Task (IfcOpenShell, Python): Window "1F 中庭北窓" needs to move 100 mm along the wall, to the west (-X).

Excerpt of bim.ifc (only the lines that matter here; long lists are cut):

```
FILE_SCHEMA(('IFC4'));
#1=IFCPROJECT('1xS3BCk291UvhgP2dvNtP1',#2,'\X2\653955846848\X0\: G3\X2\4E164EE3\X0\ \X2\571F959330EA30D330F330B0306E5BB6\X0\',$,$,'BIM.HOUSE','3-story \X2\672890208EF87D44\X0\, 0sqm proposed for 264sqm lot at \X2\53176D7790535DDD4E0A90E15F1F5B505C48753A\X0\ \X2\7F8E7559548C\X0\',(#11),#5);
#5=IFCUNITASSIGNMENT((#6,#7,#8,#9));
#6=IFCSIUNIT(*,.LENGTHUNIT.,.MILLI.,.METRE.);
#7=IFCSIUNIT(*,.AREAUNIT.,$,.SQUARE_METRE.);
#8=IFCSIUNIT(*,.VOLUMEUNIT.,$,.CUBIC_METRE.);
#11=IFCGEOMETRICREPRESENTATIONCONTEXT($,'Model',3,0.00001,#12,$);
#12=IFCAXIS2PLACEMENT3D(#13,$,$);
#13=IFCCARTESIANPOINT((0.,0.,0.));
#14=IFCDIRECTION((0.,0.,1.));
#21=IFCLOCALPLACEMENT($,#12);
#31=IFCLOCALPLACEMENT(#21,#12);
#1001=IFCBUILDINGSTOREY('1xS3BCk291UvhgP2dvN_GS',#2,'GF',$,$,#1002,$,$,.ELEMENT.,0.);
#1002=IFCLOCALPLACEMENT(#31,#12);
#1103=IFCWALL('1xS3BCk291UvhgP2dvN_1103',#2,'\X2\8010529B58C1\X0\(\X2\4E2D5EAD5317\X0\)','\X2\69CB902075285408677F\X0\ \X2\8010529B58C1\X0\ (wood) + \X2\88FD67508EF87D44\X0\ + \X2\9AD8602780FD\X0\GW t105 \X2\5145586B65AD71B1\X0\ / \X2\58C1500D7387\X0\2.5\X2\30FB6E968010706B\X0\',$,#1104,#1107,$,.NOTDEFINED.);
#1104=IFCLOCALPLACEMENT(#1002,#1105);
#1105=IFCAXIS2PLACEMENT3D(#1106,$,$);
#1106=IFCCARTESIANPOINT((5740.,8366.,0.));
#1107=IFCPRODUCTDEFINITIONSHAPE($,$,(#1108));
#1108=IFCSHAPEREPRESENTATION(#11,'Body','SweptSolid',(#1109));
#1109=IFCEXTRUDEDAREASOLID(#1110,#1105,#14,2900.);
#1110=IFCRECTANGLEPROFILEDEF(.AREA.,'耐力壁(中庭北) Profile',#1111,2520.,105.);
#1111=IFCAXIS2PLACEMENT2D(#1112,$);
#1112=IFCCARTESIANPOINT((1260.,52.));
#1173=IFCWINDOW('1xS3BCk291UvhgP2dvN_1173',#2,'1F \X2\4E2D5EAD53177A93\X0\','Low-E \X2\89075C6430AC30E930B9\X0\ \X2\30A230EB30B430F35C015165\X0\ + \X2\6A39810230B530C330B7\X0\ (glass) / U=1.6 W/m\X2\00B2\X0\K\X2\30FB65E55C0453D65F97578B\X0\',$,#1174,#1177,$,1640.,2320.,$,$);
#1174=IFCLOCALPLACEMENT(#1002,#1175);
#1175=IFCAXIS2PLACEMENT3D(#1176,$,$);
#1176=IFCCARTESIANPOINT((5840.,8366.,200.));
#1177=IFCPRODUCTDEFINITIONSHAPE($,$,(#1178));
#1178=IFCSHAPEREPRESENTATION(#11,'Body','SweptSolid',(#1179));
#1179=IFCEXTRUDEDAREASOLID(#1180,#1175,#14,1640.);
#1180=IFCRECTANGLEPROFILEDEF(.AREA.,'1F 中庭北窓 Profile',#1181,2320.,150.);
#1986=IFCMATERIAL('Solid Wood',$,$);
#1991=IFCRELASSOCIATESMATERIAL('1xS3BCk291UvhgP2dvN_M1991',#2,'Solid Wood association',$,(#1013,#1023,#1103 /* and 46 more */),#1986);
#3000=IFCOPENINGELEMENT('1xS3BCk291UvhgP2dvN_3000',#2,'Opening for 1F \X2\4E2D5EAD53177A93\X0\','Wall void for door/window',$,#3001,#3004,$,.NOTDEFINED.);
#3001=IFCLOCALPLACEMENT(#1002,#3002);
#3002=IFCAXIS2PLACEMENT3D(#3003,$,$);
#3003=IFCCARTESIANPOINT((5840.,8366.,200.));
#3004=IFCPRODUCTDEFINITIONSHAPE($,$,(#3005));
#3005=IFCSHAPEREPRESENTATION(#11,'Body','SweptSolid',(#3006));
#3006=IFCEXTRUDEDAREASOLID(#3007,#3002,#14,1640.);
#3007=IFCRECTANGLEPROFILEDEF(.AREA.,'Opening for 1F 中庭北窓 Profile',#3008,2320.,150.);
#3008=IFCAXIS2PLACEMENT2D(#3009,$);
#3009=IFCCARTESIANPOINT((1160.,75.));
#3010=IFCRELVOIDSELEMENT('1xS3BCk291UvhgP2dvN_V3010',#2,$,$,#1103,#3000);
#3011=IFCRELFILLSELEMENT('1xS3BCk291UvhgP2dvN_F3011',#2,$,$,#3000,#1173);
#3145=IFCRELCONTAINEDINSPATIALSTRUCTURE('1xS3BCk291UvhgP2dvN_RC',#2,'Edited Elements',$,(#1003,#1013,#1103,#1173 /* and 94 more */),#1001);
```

```python
import ifcopenshell
import ifcopenshell.api.geometry
import ifcopenshell.util.placement

model = ifcopenshell.open("bim.ifc")

window = model.by_guid("1xS3BCk291UvhgP2dvN_1173")
opening = window.FillsVoids[0].RelatingOpeningElement
wall = opening.VoidsElements[0].RelatingBuildingElement

wall_matrix = ifcopenshell.util.placement.get_local_placement(wall.ObjectPlacement)
shift = wall_matrix[:3, 0] * -100.0
before = ifcopenshell.util.placement.get_local_placement(window.ObjectPlacement)[:3, 3].copy()

# The window is not placed relative to its opening, so move both.
for product in (opening, window):
    matrix = ifcopenshell.util.placement.get_local_placement(product.ObjectPlacement)
    matrix[:3, 3] += shift
    ifcopenshell.api.geometry.edit_object_placement(model, product=product, matrix=matrix, is_si=False)

after = ifcopenshell.util.placement.get_local_placement(window.ObjectPlacement)[:3, 3]
print("window moved by", (after - before).round(3) + 0.0)

model.write("bim-out.ifc")
```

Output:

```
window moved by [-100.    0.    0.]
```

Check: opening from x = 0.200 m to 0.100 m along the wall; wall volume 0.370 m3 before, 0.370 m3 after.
